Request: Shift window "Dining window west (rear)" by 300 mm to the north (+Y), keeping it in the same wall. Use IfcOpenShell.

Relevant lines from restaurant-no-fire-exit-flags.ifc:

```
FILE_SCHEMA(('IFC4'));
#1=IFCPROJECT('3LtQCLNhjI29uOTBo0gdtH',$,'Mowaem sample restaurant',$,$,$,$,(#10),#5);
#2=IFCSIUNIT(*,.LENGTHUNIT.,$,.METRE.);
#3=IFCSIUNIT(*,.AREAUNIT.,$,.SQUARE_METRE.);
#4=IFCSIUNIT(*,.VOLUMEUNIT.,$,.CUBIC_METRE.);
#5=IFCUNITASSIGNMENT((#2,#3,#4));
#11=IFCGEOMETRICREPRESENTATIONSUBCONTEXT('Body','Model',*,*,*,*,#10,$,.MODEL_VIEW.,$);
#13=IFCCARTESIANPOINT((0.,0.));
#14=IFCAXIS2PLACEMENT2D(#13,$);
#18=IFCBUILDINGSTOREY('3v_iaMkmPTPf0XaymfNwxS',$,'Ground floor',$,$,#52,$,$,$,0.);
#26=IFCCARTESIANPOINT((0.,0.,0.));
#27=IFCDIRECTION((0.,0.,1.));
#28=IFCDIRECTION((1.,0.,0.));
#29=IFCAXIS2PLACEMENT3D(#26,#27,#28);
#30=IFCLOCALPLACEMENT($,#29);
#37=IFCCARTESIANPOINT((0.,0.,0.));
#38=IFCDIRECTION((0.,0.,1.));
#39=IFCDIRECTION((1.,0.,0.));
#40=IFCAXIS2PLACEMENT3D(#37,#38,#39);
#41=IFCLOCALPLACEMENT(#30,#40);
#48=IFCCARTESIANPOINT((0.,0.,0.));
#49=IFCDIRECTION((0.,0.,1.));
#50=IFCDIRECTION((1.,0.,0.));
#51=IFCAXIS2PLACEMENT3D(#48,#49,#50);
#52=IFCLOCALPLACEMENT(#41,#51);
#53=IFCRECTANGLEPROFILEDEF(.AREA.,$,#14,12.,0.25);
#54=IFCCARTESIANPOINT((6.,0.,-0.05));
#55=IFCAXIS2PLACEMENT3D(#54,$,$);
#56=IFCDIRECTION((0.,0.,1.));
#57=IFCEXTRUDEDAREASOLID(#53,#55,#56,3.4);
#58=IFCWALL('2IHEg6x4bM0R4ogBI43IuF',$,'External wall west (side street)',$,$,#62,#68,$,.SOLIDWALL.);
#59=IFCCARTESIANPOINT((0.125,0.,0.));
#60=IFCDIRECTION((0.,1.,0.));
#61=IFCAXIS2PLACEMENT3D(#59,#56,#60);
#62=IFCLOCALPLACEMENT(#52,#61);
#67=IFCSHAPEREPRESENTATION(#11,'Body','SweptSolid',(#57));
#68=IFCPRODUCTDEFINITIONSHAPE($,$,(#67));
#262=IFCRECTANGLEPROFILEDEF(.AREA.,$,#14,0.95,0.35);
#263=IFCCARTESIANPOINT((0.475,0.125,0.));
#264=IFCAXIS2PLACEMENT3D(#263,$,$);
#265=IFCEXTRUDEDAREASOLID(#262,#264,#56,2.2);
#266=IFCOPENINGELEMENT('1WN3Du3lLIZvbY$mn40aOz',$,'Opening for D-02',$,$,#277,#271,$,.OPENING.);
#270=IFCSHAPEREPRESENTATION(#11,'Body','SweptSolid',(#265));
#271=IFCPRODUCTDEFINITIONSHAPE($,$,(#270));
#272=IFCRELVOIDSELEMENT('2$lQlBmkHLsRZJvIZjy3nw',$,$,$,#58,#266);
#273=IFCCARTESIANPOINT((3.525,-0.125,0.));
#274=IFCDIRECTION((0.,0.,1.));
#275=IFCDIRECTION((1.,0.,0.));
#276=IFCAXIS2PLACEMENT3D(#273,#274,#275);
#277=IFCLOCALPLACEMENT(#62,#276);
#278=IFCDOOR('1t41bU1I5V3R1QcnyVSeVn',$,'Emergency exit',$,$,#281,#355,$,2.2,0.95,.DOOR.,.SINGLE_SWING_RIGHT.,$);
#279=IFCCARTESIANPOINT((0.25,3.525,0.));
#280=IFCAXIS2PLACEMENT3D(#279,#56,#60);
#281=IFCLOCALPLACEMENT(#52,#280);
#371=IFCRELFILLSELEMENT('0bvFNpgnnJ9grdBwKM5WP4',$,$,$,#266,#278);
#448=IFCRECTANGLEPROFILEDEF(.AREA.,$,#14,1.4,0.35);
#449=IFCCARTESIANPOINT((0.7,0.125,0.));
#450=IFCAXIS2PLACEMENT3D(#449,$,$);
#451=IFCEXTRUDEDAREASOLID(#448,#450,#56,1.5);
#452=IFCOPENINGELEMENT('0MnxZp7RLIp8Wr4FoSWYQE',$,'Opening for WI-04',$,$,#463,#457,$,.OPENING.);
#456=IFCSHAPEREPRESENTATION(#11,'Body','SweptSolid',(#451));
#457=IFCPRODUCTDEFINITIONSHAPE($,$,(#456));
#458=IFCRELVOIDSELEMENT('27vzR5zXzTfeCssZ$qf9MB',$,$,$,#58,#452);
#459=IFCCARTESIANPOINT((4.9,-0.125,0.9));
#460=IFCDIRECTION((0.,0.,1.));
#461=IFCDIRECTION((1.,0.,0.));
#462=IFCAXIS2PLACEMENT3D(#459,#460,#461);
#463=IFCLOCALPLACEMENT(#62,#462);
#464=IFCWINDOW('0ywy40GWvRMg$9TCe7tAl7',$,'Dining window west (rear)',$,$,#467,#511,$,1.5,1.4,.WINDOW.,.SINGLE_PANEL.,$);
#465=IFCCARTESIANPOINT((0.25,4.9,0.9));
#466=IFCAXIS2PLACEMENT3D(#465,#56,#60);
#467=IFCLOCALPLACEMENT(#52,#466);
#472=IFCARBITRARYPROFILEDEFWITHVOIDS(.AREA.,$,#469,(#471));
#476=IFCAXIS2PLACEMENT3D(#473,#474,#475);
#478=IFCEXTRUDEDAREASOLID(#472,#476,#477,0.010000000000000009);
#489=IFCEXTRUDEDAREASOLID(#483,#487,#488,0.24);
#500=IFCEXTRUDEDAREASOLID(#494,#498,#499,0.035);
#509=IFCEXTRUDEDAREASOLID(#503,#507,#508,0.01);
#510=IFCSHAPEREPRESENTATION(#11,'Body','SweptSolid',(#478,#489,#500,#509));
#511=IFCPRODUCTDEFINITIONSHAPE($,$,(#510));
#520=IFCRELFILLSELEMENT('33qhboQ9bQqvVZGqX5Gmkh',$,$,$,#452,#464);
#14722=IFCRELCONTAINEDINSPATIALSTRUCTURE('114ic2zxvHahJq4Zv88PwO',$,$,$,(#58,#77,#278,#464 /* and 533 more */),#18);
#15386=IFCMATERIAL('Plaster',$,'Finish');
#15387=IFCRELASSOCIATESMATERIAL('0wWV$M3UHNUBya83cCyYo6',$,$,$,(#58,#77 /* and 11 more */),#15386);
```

```python
import ifcopenshell
import ifcopenshell.api.geometry
import ifcopenshell.util.placement
import ifcopenshell.util.unit

model = ifcopenshell.open("restaurant-no-fire-exit-flags.ifc")
unit_scale = ifcopenshell.util.unit.calculate_unit_scale(model)

window = model.by_guid("0ywy40GWvRMg$9TCe7tAl7")
opening = window.FillsVoids[0].RelatingOpeningElement
wall = opening.VoidsElements[0].RelatingBuildingElement

wall_matrix = ifcopenshell.util.placement.get_local_placement(wall.ObjectPlacement)
shift = wall_matrix[:3, 0] * 0.3 / unit_scale
before = ifcopenshell.util.placement.get_local_placement(window.ObjectPlacement)[:3, 3].copy()

# The window is not placed relative to its opening, so move both.
for product in (opening, window):
    matrix = ifcopenshell.util.placement.get_local_placement(product.ObjectPlacement)
    matrix[:3, 3] += shift
    ifcopenshell.api.geometry.edit_object_placement(model, product=product, matrix=matrix, is_si=False)

after = ifcopenshell.util.placement.get_local_placement(window.ObjectPlacement)[:3, 3]
print("window moved by", (after - before).round(3) + 0.0)

model.write("restaurant-no-fire-exit-flags_updated.ifc")
```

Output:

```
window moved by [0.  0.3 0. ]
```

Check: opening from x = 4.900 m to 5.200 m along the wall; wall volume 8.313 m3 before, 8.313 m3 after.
